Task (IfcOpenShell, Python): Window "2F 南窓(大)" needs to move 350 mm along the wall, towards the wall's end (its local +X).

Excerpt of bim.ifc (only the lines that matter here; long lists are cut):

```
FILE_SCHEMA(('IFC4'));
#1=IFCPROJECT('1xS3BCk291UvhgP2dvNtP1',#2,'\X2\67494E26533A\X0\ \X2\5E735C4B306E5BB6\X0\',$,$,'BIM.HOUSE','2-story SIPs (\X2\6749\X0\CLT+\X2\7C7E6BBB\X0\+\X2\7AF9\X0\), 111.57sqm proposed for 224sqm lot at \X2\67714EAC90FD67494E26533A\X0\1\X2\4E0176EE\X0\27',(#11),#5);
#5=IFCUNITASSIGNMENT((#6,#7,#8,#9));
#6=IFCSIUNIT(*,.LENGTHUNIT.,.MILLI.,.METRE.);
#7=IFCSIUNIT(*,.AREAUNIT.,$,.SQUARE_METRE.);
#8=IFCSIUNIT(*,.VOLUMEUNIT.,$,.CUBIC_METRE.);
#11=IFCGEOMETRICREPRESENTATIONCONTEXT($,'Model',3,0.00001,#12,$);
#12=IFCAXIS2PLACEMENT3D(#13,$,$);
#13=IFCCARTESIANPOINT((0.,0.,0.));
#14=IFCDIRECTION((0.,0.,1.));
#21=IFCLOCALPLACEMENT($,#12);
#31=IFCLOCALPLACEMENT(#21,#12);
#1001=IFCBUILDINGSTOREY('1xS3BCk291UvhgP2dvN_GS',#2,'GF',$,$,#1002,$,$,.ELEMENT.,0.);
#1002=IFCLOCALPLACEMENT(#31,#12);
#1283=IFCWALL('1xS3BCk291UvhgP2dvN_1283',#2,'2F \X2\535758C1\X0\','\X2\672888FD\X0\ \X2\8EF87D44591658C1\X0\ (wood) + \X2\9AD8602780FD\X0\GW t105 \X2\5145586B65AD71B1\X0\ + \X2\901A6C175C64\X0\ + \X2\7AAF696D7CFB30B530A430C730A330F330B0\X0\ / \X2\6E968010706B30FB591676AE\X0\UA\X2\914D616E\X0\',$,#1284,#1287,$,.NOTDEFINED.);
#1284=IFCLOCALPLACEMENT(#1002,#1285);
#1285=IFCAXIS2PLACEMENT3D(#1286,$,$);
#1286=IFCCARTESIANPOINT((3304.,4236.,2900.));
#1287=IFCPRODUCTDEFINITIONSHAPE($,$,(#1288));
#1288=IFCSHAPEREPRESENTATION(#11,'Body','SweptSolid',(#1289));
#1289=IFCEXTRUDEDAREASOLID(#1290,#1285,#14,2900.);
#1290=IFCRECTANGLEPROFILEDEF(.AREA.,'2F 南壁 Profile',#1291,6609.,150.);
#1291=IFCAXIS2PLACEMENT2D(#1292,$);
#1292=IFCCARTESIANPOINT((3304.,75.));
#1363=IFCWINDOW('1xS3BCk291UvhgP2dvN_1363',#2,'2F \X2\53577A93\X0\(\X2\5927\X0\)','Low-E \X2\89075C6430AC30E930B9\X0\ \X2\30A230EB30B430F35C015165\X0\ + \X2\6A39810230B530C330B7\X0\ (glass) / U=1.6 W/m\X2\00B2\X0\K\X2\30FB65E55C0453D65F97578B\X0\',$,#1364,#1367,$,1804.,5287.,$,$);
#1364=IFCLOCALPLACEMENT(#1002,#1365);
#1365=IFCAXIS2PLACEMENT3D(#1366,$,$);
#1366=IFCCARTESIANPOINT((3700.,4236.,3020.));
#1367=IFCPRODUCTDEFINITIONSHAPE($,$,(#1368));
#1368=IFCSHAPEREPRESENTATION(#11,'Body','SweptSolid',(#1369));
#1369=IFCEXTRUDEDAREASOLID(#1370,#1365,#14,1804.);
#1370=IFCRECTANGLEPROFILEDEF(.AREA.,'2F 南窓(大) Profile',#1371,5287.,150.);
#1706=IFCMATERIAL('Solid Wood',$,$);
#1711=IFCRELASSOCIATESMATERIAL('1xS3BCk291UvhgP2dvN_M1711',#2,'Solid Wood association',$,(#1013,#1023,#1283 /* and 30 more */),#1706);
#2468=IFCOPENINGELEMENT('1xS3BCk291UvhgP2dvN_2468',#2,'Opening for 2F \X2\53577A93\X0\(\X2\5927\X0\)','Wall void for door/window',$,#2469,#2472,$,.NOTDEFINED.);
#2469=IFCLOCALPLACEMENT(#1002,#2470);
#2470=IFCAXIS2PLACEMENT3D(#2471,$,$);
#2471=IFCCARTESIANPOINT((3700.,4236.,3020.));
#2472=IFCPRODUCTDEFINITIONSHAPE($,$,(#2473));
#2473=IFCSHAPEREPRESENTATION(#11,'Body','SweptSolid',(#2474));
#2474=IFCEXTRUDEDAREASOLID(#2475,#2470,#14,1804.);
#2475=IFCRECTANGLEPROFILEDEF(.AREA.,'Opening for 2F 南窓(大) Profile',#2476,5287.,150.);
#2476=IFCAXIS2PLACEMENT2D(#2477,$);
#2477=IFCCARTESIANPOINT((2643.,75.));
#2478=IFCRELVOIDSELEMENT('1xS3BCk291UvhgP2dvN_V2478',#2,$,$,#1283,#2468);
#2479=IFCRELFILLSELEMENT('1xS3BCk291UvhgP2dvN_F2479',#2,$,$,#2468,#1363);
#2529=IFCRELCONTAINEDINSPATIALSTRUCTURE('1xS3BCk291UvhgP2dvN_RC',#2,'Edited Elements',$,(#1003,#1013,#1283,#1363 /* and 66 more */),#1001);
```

```python
import ifcopenshell
import ifcopenshell.api.geometry
import ifcopenshell.util.placement

model = ifcopenshell.open("bim.ifc")

window = model.by_id(1363)
opening = window.FillsVoids[0].RelatingOpeningElement
wall = opening.VoidsElements[0].RelatingBuildingElement

wall_matrix = ifcopenshell.util.placement.get_local_placement(wall.ObjectPlacement)
shift = wall_matrix[:3, 0] * 350.0
before = ifcopenshell.util.placement.get_local_placement(window.ObjectPlacement)[:3, 3].copy()

# The window is not placed relative to its opening, so move both.
for product in (opening, window):
    matrix = ifcopenshell.util.placement.get_local_placement(product.ObjectPlacement)
    matrix[:3, 3] += shift
    ifcopenshell.api.geometry.edit_object_placement(model, product=product, matrix=matrix, is_si=False)

after = ifcopenshell.util.placement.get_local_placement(window.ObjectPlacement)[:3, 3]
print("window moved by", (after - before).round(3) + 0.0)

model.write("bim_v2.ifc")
```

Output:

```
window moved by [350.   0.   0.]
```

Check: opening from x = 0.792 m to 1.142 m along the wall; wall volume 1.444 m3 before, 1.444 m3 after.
